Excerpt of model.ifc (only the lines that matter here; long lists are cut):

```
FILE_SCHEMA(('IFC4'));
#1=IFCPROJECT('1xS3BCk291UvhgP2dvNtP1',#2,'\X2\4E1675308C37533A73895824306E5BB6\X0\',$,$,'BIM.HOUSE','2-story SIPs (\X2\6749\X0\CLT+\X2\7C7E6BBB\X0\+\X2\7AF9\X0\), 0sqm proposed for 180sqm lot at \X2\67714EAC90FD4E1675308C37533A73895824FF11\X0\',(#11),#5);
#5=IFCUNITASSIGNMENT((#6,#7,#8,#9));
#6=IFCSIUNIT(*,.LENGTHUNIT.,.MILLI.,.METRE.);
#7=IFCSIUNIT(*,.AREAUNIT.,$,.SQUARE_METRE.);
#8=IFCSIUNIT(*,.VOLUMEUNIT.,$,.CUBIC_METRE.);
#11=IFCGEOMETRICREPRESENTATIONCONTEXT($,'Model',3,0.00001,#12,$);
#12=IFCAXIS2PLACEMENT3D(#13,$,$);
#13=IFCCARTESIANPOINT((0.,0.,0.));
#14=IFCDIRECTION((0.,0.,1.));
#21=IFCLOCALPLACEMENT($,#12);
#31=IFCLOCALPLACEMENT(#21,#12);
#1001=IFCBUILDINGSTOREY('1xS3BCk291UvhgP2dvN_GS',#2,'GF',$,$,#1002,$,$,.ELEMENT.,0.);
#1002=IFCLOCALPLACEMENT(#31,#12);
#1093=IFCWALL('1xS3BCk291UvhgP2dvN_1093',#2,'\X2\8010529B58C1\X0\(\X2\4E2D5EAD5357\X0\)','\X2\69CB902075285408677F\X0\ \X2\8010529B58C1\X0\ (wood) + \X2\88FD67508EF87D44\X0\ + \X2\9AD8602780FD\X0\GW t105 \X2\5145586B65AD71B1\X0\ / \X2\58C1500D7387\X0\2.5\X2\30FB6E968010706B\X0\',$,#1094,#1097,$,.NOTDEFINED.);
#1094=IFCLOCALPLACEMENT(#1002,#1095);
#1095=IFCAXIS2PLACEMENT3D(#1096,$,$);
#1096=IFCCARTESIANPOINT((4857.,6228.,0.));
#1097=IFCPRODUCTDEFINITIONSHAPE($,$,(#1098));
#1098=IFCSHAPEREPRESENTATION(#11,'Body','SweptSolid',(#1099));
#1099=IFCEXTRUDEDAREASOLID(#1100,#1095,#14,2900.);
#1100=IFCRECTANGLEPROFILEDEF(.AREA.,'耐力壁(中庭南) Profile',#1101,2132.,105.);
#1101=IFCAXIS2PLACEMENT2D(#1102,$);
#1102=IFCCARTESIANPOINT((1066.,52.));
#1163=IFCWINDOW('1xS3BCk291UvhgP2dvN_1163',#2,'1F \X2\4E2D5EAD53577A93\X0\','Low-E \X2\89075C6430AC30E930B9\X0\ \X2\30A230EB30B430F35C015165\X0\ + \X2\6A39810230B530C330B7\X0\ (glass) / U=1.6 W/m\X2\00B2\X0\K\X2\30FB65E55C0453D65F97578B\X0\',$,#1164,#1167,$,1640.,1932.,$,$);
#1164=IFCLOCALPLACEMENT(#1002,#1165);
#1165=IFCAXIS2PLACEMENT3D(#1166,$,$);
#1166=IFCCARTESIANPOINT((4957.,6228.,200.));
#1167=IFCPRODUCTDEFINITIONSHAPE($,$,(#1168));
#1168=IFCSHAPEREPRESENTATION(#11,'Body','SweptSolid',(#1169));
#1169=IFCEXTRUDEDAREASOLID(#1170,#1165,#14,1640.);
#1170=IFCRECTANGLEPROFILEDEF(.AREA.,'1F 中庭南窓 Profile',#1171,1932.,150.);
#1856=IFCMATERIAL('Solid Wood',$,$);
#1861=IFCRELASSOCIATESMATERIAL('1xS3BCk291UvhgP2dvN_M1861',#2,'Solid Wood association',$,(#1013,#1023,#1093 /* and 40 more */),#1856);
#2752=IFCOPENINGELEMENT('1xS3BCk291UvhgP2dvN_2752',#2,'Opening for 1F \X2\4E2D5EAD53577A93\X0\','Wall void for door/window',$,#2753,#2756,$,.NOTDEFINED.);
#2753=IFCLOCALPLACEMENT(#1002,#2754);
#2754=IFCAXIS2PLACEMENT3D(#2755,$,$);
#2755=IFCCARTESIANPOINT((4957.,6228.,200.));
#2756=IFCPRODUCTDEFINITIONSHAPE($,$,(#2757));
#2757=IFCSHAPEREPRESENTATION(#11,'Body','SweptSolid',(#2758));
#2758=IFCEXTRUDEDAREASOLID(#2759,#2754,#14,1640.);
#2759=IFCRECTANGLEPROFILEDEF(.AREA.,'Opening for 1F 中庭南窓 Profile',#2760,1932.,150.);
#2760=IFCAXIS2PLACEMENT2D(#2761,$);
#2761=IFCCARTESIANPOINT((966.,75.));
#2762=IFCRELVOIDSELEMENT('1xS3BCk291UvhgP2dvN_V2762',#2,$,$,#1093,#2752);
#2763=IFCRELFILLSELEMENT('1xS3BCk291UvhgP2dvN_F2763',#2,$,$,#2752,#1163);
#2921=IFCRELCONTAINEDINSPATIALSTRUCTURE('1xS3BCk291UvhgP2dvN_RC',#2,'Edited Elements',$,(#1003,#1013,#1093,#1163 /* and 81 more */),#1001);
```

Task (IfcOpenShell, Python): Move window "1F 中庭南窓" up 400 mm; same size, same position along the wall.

```python
import numpy as np
import ifcopenshell
import ifcopenshell.api.geometry
import ifcopenshell.util.placement
import ifcopenshell.util.unit

model = ifcopenshell.open("model.ifc")
unit_scale = ifcopenshell.util.unit.calculate_unit_scale(model)

window = model.by_id(1163)
opening = window.FillsVoids[0].RelatingOpeningElement
dz = 0.4 / unit_scale

shift = np.array([0.0, 0.0, dz])
# The window is not placed relative to its opening, so move both.
for product in (opening, window):
    matrix = ifcopenshell.util.placement.get_local_placement(product.ObjectPlacement)
    matrix[:3, 3] += shift
    ifcopenshell.api.geometry.edit_object_placement(model, product=product, matrix=matrix, is_si=False)

print(f"moved by {dz * unit_scale:+.3f} m")

model.write("model-out.ifc")
```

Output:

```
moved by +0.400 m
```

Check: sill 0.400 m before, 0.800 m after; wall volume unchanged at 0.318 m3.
